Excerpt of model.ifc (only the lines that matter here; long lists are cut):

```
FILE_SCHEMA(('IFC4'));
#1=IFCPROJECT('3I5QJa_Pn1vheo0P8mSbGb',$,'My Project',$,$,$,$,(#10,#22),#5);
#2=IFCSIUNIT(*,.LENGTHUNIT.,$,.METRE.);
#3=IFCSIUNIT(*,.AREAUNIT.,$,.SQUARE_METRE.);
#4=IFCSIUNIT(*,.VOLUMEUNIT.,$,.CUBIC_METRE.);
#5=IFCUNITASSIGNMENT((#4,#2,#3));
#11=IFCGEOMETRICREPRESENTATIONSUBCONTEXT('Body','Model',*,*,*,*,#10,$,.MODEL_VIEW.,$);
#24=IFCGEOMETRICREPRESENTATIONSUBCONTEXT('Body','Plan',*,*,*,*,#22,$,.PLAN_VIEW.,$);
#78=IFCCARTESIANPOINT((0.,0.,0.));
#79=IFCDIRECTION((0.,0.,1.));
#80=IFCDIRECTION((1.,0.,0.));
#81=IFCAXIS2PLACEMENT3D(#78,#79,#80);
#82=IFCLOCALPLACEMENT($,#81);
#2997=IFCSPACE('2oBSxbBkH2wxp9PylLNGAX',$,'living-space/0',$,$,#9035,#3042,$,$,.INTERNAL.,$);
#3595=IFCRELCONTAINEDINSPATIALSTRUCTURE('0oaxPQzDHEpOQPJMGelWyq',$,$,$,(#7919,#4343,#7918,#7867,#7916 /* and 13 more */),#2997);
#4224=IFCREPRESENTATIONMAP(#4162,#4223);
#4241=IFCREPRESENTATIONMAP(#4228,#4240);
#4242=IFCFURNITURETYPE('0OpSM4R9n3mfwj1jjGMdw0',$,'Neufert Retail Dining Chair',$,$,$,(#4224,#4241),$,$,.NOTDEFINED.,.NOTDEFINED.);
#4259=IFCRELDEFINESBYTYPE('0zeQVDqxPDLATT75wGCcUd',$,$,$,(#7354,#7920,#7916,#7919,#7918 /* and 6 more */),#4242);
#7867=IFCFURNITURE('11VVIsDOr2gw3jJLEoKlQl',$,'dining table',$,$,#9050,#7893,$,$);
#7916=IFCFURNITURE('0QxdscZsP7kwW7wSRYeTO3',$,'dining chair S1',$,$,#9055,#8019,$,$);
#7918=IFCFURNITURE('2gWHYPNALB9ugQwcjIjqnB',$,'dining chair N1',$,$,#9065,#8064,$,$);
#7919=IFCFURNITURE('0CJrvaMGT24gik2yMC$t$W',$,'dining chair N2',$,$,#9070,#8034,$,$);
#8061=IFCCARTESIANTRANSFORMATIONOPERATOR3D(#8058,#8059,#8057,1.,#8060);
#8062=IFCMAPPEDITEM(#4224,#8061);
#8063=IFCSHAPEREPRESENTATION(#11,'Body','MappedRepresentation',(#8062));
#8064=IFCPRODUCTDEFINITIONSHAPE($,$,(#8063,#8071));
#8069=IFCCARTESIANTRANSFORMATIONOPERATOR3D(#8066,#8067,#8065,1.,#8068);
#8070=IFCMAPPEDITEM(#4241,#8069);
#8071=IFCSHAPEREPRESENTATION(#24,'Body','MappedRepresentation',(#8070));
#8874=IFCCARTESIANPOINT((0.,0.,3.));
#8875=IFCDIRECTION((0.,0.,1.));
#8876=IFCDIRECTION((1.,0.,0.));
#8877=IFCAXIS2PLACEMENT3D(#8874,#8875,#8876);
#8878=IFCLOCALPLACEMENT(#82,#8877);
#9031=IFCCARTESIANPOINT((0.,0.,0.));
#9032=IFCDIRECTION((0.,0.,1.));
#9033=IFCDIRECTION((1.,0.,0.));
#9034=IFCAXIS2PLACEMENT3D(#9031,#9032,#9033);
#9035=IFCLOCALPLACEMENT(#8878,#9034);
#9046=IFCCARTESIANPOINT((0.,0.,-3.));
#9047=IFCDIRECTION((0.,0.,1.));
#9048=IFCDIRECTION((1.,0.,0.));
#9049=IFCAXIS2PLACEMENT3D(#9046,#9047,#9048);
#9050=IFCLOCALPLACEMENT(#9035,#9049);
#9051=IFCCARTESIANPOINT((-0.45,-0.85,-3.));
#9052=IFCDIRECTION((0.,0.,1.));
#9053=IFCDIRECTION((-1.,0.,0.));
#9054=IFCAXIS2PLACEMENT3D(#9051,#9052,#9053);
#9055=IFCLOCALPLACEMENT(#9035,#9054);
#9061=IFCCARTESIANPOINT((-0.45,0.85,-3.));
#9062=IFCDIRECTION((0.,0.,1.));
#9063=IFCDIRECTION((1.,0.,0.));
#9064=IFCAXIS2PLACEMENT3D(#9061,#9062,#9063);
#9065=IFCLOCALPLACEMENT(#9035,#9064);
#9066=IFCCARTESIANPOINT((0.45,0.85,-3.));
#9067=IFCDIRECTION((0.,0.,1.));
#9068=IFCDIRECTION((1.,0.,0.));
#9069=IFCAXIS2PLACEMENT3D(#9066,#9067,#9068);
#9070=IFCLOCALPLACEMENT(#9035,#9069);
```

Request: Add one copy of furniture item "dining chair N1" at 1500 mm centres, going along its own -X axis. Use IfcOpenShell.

```python
import ifcopenshell
import ifcopenshell.api.geometry
import ifcopenshell.api.root
import ifcopenshell.util.element
import ifcopenshell.util.placement
import ifcopenshell.util.unit

model = ifcopenshell.open("model.ifc")
unit_scale = ifcopenshell.util.unit.calculate_unit_scale(model)

source = model.by_id(7918)
base = ifcopenshell.util.placement.get_local_placement(source.ObjectPlacement)
step = -base[:3, 0] * 1.5 / unit_scale

for i in range(1, 2):
    copy = ifcopenshell.api.root.copy_class(model, product=source)
    copy.Representation = ifcopenshell.util.element.copy_deep(
        model, source.Representation, exclude=["IfcGeometricRepresentationContext", "IfcRepresentationMap"]
    )
    matrix = base.copy()
    matrix[:3, 3] += i * step
    print("added at", matrix[:3, 3].round(3) + 0.0)
    ifcopenshell.api.geometry.edit_object_placement(model, product=copy, matrix=matrix, is_si=False)

model.write("model_updated.ifc")
```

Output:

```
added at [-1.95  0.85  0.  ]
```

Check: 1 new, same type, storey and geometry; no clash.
